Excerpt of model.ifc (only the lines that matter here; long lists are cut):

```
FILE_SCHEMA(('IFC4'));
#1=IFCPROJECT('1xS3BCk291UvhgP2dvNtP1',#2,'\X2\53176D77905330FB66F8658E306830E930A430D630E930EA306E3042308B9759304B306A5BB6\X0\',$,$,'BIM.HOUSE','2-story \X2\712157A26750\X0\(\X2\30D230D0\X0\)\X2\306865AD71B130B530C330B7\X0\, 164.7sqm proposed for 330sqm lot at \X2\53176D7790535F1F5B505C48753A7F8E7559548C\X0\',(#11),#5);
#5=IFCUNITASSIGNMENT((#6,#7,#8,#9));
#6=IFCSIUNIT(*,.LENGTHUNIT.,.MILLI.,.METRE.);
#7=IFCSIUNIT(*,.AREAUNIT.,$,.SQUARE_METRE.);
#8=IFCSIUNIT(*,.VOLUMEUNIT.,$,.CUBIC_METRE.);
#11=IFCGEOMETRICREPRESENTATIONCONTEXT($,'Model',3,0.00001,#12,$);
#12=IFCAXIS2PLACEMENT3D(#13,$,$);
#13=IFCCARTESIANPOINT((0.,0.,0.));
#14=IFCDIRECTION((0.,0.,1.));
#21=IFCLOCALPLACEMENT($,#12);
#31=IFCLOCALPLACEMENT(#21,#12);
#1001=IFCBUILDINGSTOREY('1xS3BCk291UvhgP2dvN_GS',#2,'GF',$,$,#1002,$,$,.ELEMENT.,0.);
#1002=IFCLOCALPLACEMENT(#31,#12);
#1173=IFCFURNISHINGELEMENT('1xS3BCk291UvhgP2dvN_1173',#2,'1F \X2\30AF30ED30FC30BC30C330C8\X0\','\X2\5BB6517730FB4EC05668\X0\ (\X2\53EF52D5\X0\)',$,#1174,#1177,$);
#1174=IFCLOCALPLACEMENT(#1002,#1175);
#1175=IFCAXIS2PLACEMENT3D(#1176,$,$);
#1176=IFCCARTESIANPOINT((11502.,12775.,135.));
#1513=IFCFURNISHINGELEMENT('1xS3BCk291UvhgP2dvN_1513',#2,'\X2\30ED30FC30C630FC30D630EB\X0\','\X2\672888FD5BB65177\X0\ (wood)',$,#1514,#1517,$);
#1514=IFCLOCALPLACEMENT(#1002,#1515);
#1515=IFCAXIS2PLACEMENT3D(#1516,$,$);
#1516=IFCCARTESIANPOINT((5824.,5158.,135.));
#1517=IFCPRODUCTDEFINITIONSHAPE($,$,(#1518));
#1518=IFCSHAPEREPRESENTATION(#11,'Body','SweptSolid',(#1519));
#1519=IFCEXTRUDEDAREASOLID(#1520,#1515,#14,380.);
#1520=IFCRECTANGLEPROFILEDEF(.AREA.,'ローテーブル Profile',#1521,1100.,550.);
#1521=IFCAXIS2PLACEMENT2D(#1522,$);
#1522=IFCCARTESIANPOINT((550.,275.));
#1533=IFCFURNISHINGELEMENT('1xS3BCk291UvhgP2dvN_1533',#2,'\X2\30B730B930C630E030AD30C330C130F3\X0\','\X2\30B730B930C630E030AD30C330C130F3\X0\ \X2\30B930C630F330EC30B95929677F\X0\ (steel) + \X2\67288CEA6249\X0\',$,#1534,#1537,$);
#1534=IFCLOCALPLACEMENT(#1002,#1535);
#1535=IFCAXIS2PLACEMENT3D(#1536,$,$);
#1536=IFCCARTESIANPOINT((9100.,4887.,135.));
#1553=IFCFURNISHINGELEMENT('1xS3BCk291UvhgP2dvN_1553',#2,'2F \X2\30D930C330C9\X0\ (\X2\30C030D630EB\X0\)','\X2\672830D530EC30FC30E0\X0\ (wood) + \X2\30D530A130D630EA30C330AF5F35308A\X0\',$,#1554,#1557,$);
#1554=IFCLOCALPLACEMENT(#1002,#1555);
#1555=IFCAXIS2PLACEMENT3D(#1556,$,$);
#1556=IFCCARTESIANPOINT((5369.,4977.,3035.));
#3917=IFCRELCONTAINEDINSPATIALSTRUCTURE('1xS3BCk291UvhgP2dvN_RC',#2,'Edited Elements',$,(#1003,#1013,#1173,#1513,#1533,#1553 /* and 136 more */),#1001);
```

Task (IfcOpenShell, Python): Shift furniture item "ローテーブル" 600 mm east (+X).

```python
import ifcopenshell
import ifcopenshell.api.geometry
import ifcopenshell.util.placement
import ifcopenshell.util.unit

model = ifcopenshell.open("model.ifc")
unit_scale = ifcopenshell.util.unit.calculate_unit_scale(model)

item = model.by_guid("1xS3BCk291UvhgP2dvN_1513")
matrix = ifcopenshell.util.placement.get_local_placement(item.ObjectPlacement)
matrix[0, 3] += 0.6 / unit_scale
ifcopenshell.api.geometry.edit_object_placement(model, product=item, matrix=matrix, is_si=False)

print(ifcopenshell.util.placement.get_local_placement(item.ObjectPlacement).round(3) + 0.0)

model.write("model_v2.ifc")
```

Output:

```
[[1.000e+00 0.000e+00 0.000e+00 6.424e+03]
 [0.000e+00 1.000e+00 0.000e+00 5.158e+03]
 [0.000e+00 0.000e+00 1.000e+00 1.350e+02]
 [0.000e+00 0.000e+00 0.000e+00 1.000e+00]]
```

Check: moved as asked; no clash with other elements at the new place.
